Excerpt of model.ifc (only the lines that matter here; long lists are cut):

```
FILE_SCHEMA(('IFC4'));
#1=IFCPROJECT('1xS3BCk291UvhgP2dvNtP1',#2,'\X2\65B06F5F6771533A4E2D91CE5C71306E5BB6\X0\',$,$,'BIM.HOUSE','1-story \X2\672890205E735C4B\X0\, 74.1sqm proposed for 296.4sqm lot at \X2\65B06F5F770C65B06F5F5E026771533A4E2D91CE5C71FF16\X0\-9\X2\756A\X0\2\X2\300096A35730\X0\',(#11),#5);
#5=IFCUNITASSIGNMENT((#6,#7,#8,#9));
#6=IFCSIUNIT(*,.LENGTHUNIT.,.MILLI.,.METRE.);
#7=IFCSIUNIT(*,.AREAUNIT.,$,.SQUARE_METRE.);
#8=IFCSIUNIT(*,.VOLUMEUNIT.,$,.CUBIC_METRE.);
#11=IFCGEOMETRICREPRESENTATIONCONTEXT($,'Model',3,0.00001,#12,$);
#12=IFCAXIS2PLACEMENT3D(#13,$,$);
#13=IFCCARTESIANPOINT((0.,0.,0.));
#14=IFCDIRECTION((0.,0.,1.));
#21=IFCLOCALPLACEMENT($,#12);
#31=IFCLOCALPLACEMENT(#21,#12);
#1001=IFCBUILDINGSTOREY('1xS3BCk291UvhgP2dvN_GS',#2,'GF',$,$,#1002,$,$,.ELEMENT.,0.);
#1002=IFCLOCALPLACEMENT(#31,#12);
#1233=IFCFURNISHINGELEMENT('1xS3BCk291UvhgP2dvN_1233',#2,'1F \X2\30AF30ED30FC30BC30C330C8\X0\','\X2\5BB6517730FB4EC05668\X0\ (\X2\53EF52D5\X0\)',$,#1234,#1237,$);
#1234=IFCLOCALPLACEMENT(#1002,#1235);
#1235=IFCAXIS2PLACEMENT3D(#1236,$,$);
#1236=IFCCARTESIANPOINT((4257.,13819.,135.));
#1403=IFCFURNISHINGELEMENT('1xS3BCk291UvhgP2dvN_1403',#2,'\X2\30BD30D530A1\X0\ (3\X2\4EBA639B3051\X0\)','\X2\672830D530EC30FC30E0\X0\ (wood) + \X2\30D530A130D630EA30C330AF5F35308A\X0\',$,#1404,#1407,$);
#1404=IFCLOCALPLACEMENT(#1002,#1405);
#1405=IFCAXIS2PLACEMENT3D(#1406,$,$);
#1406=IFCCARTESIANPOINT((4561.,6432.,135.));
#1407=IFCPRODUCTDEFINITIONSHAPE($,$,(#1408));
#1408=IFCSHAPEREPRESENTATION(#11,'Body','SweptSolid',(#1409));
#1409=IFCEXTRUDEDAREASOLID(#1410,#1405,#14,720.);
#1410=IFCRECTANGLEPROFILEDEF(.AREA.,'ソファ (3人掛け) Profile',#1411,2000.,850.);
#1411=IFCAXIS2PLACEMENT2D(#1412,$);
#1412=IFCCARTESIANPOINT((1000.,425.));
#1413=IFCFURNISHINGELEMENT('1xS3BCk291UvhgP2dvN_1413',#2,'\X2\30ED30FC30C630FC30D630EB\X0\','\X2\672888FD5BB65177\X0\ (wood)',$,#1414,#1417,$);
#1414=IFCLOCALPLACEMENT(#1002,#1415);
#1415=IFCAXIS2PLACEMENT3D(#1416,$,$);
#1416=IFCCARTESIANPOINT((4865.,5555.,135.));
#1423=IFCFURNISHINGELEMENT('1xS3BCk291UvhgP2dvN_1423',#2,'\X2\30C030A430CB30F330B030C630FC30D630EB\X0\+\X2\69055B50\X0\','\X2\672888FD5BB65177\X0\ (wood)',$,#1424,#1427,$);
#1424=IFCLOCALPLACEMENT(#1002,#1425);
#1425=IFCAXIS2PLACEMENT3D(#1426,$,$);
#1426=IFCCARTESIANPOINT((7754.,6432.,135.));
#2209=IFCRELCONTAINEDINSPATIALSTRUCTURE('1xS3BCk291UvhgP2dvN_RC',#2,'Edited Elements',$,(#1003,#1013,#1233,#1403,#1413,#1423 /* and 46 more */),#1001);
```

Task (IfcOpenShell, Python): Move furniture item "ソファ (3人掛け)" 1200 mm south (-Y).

```python
import ifcopenshell
import ifcopenshell.api.geometry
import ifcopenshell.util.placement
import ifcopenshell.util.unit

model = ifcopenshell.open("model.ifc")
unit_scale = ifcopenshell.util.unit.calculate_unit_scale(model)

item = model.by_guid("1xS3BCk291UvhgP2dvN_1403")
matrix = ifcopenshell.util.placement.get_local_placement(item.ObjectPlacement)
matrix[1, 3] -= 1.2 / unit_scale
ifcopenshell.api.geometry.edit_object_placement(model, product=item, matrix=matrix, is_si=False)

print(ifcopenshell.util.placement.get_local_placement(item.ObjectPlacement).round(3) + 0.0)

model.write("model_edited.ifc")
```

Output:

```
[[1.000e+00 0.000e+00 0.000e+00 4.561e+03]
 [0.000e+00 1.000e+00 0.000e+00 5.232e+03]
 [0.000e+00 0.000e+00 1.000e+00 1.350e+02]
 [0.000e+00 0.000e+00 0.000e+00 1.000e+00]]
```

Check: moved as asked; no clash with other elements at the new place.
